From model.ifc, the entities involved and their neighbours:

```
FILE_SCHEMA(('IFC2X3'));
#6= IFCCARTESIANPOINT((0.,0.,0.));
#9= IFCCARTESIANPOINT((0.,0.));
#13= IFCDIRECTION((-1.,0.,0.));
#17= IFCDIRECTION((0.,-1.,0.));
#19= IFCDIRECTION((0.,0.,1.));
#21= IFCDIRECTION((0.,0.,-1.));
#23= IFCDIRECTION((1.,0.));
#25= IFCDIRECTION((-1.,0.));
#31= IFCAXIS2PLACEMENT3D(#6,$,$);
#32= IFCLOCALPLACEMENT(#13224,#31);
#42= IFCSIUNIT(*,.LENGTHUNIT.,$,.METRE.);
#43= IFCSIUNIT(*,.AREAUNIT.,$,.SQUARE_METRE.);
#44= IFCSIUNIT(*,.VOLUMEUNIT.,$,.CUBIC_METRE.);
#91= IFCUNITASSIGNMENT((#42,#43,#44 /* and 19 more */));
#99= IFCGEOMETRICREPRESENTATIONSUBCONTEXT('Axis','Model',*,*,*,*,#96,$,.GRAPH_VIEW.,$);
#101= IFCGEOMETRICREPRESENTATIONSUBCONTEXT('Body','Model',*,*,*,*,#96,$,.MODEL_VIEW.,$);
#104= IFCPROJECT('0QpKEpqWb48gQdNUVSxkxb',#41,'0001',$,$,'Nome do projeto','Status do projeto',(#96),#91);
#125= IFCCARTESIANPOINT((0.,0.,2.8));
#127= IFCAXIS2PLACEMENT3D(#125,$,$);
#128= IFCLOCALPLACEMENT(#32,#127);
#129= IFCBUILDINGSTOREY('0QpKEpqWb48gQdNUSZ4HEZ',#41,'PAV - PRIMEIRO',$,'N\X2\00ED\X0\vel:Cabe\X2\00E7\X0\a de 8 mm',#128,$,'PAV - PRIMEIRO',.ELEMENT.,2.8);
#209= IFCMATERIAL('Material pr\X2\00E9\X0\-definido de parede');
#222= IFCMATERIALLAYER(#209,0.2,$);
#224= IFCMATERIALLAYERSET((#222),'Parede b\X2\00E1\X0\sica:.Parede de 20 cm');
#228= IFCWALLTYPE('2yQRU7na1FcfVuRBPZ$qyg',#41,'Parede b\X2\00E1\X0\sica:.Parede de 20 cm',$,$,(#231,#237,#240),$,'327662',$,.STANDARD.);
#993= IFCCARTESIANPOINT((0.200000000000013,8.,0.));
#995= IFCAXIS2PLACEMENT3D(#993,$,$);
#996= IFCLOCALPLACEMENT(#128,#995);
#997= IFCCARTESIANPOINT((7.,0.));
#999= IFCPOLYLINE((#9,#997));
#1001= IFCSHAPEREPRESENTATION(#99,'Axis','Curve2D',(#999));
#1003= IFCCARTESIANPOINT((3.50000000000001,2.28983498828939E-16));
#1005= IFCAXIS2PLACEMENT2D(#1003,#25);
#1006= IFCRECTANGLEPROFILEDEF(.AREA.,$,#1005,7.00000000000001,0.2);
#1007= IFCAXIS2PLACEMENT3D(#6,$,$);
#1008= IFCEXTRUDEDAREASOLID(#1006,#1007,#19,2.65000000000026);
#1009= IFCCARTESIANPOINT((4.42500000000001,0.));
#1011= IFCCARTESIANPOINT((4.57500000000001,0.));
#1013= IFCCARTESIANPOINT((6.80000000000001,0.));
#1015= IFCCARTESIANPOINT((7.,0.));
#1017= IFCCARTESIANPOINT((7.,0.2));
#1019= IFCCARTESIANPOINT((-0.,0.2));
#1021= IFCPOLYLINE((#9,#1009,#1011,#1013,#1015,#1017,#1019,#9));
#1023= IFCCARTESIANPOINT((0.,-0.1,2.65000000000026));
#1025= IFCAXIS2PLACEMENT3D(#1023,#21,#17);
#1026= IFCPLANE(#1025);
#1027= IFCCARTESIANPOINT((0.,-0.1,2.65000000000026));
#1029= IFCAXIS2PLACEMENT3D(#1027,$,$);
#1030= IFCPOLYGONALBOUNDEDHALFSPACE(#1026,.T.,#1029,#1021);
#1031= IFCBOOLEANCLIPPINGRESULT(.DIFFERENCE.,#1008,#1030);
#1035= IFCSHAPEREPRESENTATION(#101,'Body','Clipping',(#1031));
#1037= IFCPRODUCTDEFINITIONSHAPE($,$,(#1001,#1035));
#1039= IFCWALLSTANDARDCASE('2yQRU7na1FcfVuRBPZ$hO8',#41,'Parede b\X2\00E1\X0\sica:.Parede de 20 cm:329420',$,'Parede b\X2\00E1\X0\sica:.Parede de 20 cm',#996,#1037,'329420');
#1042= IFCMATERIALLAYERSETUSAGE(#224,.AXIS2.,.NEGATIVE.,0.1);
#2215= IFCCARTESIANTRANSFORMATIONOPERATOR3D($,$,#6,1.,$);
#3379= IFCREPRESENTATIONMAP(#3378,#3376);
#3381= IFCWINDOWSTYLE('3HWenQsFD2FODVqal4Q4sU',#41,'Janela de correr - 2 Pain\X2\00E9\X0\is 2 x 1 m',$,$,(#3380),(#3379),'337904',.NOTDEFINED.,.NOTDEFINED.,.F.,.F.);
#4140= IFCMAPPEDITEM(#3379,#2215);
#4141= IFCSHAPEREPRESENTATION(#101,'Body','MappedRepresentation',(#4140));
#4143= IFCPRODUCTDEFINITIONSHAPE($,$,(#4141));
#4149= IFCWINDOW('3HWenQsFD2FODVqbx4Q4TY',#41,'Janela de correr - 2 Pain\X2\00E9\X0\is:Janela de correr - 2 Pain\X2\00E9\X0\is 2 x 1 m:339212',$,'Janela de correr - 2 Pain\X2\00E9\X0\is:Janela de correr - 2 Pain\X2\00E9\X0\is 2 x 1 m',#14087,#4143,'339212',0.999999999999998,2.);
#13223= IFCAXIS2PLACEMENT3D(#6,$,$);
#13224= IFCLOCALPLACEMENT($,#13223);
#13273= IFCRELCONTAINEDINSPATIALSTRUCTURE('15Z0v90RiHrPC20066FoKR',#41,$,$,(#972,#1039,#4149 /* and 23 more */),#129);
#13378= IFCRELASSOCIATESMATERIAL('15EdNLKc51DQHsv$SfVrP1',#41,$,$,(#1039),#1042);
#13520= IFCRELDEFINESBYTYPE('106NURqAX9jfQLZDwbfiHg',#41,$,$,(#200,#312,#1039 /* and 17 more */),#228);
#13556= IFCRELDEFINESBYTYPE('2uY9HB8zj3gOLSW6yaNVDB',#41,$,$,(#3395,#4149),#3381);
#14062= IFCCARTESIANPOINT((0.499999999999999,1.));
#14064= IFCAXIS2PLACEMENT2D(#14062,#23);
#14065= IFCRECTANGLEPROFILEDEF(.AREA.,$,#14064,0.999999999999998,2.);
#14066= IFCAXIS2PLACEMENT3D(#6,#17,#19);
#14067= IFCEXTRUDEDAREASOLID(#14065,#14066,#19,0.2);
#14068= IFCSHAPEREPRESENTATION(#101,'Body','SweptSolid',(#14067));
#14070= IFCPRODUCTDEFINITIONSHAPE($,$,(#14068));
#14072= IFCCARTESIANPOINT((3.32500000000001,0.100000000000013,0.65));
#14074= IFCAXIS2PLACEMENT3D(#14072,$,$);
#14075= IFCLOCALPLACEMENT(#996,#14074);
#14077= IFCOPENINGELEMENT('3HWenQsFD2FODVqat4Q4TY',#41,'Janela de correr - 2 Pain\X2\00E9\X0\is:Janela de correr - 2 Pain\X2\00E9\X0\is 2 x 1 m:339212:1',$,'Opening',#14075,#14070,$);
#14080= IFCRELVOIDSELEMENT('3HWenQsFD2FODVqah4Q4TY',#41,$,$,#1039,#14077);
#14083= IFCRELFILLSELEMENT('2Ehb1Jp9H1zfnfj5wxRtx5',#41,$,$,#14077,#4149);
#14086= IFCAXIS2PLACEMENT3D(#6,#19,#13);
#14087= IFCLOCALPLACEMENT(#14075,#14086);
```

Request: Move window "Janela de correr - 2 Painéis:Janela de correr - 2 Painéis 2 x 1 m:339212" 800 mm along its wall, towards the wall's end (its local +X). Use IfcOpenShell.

```python
import ifcopenshell
import ifcopenshell.api.geometry
import ifcopenshell.util.placement
import ifcopenshell.util.unit

model = ifcopenshell.open("model.ifc")
unit_scale = ifcopenshell.util.unit.calculate_unit_scale(model)

window = model.by_guid("3HWenQsFD2FODVqbx4Q4TY")
opening = window.FillsVoids[0].RelatingOpeningElement
wall = opening.VoidsElements[0].RelatingBuildingElement

wall_matrix = ifcopenshell.util.placement.get_local_placement(wall.ObjectPlacement)
shift = wall_matrix[:3, 0] * 0.8 / unit_scale
before = ifcopenshell.util.placement.get_local_placement(window.ObjectPlacement)[:3, 3].copy()

# The window is placed relative to its opening, so it follows when the opening moves.
matrix = ifcopenshell.util.placement.get_local_placement(opening.ObjectPlacement)
matrix[:3, 3] += shift
ifcopenshell.api.geometry.edit_object_placement(
    model, product=opening, matrix=matrix, is_si=False, should_transform_children=True
)

after = ifcopenshell.util.placement.get_local_placement(window.ObjectPlacement)[:3, 3]
print("window moved by", (after - before).round(3) + 0.0)

model.write("model_edited.ifc")
```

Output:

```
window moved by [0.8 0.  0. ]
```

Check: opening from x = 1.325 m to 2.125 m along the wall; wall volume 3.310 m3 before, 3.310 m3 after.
